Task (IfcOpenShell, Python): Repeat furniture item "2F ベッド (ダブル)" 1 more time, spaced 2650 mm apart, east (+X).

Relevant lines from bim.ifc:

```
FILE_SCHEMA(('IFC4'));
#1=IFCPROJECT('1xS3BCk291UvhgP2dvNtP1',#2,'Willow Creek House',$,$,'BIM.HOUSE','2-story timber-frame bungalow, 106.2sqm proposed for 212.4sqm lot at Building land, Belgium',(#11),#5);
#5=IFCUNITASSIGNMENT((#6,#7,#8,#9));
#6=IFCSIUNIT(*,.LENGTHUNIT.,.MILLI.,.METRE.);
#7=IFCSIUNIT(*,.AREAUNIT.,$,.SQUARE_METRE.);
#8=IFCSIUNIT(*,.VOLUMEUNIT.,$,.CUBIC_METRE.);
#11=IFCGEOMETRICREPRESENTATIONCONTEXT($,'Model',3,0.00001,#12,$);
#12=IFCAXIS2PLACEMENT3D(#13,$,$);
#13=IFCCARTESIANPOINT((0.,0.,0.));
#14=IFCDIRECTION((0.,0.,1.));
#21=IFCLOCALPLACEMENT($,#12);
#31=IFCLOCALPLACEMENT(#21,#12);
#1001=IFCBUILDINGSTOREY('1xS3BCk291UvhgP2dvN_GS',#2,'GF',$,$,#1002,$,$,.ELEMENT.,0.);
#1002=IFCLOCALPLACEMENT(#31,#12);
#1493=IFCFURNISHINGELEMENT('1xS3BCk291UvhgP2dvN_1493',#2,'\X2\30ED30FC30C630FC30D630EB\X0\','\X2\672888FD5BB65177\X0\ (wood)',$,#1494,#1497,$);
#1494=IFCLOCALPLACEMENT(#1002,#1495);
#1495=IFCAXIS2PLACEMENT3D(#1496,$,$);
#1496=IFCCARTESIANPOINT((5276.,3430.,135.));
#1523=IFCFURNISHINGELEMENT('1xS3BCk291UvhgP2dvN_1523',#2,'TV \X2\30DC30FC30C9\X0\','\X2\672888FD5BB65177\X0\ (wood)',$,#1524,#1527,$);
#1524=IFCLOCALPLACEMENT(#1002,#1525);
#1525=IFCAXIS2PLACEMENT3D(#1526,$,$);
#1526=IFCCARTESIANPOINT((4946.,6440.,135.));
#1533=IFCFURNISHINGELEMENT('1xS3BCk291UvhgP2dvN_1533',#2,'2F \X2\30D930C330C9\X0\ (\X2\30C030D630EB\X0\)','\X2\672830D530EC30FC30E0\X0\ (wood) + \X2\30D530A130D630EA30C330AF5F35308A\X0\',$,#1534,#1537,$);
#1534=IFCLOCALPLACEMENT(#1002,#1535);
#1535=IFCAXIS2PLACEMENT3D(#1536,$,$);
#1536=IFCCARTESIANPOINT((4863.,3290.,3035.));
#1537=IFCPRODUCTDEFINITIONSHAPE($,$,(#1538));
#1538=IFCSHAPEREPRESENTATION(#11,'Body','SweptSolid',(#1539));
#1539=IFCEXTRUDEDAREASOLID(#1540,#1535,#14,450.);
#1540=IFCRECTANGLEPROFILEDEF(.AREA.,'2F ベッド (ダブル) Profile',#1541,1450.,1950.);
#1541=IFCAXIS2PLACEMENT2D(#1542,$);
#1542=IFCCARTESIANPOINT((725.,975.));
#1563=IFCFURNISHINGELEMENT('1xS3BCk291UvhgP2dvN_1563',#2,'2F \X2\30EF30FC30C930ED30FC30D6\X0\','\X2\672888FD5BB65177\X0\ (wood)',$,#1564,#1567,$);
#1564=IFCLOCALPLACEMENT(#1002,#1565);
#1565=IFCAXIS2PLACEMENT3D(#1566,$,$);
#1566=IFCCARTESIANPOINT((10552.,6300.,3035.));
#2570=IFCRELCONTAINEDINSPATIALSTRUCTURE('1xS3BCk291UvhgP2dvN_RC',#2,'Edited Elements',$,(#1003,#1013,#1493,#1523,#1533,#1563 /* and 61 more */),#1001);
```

```python
import numpy as np
import ifcopenshell
import ifcopenshell.api.geometry
import ifcopenshell.api.root
import ifcopenshell.util.element
import ifcopenshell.util.placement
import ifcopenshell.util.unit

model = ifcopenshell.open("bim.ifc")
unit_scale = ifcopenshell.util.unit.calculate_unit_scale(model)


def reuse_history(source, copy):
    """copy_class also copies each property set's owner history, people and application; keep the originals."""
    for rel in copy.IsDefinedBy:
        if rel.is_a("IfcRelDefinesByProperties") and (history := rel.RelatingPropertyDefinition.OwnerHistory):
            rel.RelatingPropertyDefinition.OwnerHistory = source.OwnerHistory
            ifcopenshell.util.element.remove_deep2(model, history)


source = model.by_guid("1xS3BCk291UvhgP2dvN_1533")
base = ifcopenshell.util.placement.get_local_placement(source.ObjectPlacement)
step = np.array([1.0, 0.0, 0.0]) * 2.65 / unit_scale

for i in range(1, 2):
    copy = ifcopenshell.api.root.copy_class(model, product=source)
    copy.Representation = ifcopenshell.util.element.copy_deep(
        model, source.Representation, exclude=["IfcGeometricRepresentationContext", "IfcRepresentationMap"]
    )
    reuse_history(source, copy)
    matrix = base.copy()
    matrix[:3, 3] += i * step
    print("added at", matrix[:3, 3].round(3) + 0.0)
    ifcopenshell.api.geometry.edit_object_placement(model, product=copy, matrix=matrix, is_si=False)

model.write("bim-out.ifc")
```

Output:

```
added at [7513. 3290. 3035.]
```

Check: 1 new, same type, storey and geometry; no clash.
